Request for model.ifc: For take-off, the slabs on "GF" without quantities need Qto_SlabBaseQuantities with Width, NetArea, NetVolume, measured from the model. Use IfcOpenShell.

First a look at what the model holds.

```python
import ifcopenshell
import ifcopenshell.util.element
import ifcopenshell.util.unit

model = ifcopenshell.open("model.ifc")
print(model.schema)
for unit_type in ("LENGTHUNIT", "AREAUNIT", "VOLUMEUNIT"):
    print(unit_type, ifcopenshell.util.unit.calculate_unit_scale(model, unit_type))
storey = next(s for s in model.by_type("IfcBuildingStorey") if s.Name == "GF")
slabs = [e for e in ifcopenshell.util.element.get_decomposition(storey) if e.is_a("IfcSlab")]
for e in sorted(slabs, key=lambda e: e.id()):
    print(e.id(), e.is_a(), e.Name, list(ifcopenshell.util.element.get_psets(e, qtos_only=True)), sep=" | ")
```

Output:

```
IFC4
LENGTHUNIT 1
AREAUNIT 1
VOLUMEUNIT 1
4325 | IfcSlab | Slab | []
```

```python
import ifcopenshell
import ifcopenshell.api.pset
import ifcopenshell.geom
import ifcopenshell.util.element
import ifcopenshell.util.shape
import ifcopenshell.util.unit

model = ifcopenshell.open("model.ifc")
unit_scale = ifcopenshell.util.unit.calculate_unit_scale(model)
area_scale = ifcopenshell.util.unit.calculate_unit_scale(model, "AREAUNIT")
volume_scale = ifcopenshell.util.unit.calculate_unit_scale(model, "VOLUMEUNIT")
settings = ifcopenshell.geom.settings()

storey = next(s for s in model.by_type("IfcBuildingStorey") if s.Name == "GF")
slabs = [e for e in ifcopenshell.util.element.get_decomposition(storey) if e.is_a("IfcSlab")]

for e in sorted(slabs, key=lambda e: e.id()):
    if ifcopenshell.util.element.get_psets(e, qtos_only=True, should_inherit=False):
        continue
    # Geometry comes back in metres, in the element's own axes.
    shape = ifcopenshell.geom.create_shape(settings, e)
    values = {
        "Width": ifcopenshell.util.shape.get_z(shape.geometry) / unit_scale,
        "NetArea": ifcopenshell.util.shape.get_footprint_area(shape.geometry) / area_scale,
        "NetVolume": ifcopenshell.util.shape.get_volume(shape.geometry) / volume_scale,
    }
    qto = ifcopenshell.api.pset.add_qto(model, product=e, name="Qto_SlabBaseQuantities")
    ifcopenshell.api.pset.edit_qto(model, qto=qto, properties=values)
    print(e.id(), {k: round(v, 3) for k, v in values.items()})

model.write("model-out.ifc")
```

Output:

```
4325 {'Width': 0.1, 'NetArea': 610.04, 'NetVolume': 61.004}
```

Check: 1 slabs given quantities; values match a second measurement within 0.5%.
